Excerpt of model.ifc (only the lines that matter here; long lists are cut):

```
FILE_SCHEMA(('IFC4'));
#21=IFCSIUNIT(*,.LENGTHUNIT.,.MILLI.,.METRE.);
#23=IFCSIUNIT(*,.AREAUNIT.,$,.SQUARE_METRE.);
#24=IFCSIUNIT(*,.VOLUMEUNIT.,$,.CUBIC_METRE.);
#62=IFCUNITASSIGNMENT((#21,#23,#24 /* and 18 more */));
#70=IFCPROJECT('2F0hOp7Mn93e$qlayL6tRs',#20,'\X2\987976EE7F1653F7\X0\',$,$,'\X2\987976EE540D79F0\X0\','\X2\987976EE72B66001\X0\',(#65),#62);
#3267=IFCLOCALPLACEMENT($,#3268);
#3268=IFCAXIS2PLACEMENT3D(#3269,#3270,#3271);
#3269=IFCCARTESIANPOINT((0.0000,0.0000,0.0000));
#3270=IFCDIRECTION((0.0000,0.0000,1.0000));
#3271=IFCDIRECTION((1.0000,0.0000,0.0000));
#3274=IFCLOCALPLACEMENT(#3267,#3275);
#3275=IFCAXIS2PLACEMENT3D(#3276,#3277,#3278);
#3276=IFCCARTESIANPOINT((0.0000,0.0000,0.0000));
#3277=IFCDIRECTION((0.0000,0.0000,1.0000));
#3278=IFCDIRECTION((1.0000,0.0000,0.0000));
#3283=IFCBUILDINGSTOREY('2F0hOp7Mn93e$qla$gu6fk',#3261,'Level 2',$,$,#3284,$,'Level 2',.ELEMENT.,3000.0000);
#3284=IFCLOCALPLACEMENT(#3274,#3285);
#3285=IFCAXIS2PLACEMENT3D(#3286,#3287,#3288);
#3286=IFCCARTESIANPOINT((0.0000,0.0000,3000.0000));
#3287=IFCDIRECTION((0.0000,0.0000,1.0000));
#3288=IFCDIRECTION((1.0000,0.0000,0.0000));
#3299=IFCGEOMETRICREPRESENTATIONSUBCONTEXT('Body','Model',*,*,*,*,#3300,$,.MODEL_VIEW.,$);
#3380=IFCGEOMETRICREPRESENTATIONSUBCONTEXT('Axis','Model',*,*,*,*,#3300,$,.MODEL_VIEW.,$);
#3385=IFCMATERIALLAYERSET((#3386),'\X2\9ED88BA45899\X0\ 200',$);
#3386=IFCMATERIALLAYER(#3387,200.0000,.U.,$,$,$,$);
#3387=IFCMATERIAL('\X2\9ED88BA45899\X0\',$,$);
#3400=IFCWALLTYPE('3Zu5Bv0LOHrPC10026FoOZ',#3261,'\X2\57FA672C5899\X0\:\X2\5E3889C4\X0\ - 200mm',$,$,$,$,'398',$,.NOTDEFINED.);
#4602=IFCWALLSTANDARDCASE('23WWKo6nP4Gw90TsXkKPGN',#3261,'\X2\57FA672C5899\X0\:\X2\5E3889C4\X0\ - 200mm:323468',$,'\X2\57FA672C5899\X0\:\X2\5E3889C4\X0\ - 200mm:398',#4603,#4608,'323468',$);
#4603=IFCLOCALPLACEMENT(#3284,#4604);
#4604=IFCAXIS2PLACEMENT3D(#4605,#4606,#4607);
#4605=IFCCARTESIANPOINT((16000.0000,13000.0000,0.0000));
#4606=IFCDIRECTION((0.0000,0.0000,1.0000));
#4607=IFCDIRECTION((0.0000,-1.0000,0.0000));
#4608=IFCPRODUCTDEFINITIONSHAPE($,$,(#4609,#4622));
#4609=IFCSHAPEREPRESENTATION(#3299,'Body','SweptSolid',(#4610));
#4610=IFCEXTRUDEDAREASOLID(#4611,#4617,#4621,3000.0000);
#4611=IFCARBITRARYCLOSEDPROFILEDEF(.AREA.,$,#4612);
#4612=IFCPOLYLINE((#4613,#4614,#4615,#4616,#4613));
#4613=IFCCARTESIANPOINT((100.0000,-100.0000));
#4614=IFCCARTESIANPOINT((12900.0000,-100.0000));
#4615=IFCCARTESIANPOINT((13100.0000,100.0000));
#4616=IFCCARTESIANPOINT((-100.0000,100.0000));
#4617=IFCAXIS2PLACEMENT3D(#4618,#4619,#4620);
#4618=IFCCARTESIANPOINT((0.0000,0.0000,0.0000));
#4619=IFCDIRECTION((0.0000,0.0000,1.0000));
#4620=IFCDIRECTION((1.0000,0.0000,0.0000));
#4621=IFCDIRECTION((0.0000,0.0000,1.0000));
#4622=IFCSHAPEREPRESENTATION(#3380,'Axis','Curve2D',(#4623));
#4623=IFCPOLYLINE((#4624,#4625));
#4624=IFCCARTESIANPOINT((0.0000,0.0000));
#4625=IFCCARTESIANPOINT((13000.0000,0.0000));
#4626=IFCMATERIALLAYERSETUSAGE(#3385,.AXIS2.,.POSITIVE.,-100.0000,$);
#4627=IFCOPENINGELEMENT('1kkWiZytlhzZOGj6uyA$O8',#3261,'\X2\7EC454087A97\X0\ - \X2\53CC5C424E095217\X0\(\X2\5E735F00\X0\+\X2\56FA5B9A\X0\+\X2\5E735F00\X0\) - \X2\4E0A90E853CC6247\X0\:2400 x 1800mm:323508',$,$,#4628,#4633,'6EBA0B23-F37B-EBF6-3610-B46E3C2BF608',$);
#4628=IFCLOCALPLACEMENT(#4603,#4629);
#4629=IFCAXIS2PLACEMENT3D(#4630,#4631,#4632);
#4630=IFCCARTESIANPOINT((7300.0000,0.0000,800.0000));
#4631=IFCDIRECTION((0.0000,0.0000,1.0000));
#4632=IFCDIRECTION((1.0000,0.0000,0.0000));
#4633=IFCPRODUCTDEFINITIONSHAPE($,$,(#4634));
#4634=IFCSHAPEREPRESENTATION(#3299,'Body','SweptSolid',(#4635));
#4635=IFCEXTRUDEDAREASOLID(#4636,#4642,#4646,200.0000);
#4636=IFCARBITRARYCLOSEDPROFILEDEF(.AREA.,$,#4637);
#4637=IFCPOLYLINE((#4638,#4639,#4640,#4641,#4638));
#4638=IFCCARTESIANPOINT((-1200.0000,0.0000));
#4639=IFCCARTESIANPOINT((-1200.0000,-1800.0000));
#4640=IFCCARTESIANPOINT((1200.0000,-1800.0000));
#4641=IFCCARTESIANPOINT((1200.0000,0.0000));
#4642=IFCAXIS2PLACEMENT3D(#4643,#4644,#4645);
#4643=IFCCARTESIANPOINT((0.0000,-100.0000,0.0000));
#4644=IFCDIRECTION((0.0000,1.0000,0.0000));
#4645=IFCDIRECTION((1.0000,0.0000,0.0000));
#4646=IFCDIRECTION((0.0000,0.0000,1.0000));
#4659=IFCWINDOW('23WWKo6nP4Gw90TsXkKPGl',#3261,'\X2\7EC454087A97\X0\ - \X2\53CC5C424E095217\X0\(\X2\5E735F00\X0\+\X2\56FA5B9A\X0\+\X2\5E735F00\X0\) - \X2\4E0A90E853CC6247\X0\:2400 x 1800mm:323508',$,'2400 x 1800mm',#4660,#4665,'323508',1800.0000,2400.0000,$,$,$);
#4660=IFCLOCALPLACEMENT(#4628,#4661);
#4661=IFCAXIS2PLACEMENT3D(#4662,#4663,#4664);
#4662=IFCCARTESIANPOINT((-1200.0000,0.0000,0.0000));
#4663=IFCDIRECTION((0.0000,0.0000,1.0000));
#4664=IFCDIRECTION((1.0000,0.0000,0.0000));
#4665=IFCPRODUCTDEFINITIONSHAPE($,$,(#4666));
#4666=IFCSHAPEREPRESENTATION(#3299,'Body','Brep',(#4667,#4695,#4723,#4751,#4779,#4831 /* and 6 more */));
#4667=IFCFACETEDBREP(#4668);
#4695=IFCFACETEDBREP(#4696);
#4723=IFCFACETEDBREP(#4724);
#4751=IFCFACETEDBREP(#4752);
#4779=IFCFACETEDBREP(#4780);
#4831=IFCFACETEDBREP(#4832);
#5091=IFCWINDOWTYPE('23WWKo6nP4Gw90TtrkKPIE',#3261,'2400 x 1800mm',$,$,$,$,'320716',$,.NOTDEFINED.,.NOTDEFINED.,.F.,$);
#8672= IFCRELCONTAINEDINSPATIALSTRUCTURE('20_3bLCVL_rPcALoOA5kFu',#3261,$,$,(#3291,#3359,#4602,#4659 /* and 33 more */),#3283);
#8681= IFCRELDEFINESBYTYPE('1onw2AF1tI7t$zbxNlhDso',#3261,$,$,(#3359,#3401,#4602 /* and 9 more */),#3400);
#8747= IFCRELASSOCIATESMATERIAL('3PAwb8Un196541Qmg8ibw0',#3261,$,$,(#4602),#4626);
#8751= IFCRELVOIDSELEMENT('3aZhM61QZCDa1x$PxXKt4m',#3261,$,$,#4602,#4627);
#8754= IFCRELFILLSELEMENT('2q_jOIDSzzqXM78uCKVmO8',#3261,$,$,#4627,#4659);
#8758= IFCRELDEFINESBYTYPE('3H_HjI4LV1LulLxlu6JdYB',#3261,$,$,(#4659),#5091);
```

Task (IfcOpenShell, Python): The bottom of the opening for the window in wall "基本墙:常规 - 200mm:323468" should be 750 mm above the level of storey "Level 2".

```python
import numpy as np
import ifcopenshell
import ifcopenshell.api.geometry
import ifcopenshell.geom
import ifcopenshell.util.element
import ifcopenshell.util.placement
import ifcopenshell.util.shape
import ifcopenshell.util.unit

model = ifcopenshell.open("model.ifc")
unit_scale = ifcopenshell.util.unit.calculate_unit_scale(model)

window = model.by_guid("23WWKo6nP4Gw90TsXkKPGl")
opening = window.FillsVoids[0].RelatingOpeningElement
storey = ifcopenshell.util.element.get_container(window, ifc_class="IfcBuildingStorey")
level = ifcopenshell.util.placement.get_local_placement(storey.ObjectPlacement)[2, 3]

# The opening's origin need not be at the sill, so measure its lowest point.
shape = ifcopenshell.geom.create_shape(ifcopenshell.geom.settings(), opening)
bottom = ifcopenshell.util.shape.get_shape_bottom_elevation(shape, shape.geometry) / unit_scale
dz = level + 0.75 / unit_scale - bottom

shift = np.array([0.0, 0.0, dz])
# The window is placed relative to its opening, so it follows when the opening moves.
matrix = ifcopenshell.util.placement.get_local_placement(opening.ObjectPlacement)
matrix[:3, 3] += shift
ifcopenshell.api.geometry.edit_object_placement(
    model, product=opening, matrix=matrix, is_si=False, should_transform_children=True
)

print(f"moved by {dz * unit_scale:+.3f} m")

model.write("model_edited.ifc")
```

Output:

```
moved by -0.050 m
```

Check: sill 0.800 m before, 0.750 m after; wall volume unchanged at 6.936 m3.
